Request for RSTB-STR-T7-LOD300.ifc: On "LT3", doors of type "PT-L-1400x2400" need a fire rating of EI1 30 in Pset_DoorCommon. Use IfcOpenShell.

First a look at what the model holds.

```python
import ifcopenshell
import ifcopenshell.util.element

model = ifcopenshell.open("RSTB-STR-T7-LOD300.ifc")
print(model.schema)
storey = next(s for s in model.by_type("IfcBuildingStorey") if s.Name == "LT3")
doors = [e for e in ifcopenshell.util.element.get_decomposition(storey) if e.is_a("IfcDoor")]
seen = {}
for e in doors:
    element_type = ifcopenshell.util.element.get_type(e)
    key = (element_type.Name if element_type != e and element_type else None, ifcopenshell.util.element.get_pset(e, "Pset_DoorCommon", "FireRating"))
    seen[key] = seen.get(key, 0) + 1
for (name, value), count in sorted(seen.items(), key=str):
    print(count, "x", name, "|", value)
```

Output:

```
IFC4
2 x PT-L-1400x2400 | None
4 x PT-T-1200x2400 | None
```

```python
import ifcopenshell
import ifcopenshell.api.pset
import ifcopenshell.util.element

model = ifcopenshell.open("RSTB-STR-T7-LOD300.ifc")

storey = next(s for s in model.by_type("IfcBuildingStorey") if s.Name == "LT3")
doors = [e for e in ifcopenshell.util.element.get_decomposition(storey) if e.is_a("IfcDoor")]

count = 0
for e in doors:
    element_type = ifcopenshell.util.element.get_type(e)
    if element_type in (None, e) or element_type.Name != "PT-L-1400x2400":
        continue
    # add_pset returns the element's existing set when there is one.
    pset = ifcopenshell.api.pset.add_pset(model, product=e, name="Pset_DoorCommon")
    ifcopenshell.api.pset.edit_pset(model, pset=pset, properties={"FireRating": "EI1 30"})
    count += 1

print(count, "doors updated")

model.write("RSTB-STR-T7-LOD300_v2.ifc")
```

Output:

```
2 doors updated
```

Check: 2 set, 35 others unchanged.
